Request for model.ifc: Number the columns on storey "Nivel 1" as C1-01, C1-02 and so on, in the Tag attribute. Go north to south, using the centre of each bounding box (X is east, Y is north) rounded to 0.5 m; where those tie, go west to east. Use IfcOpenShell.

First a look at what the model holds.

```python
import ifcopenshell
import ifcopenshell.util.element
import ifcopenshell.util.placement

model = ifcopenshell.open("model.ifc")
print(model.schema)
storey = next(s for s in model.by_type("IfcBuildingStorey") if s.Name == "Nivel 1")
columns = [e for e in ifcopenshell.util.element.get_decomposition(storey) if e.is_a("IfcColumn")]
for e in sorted(columns, key=lambda e: e.id()):
    origin = ifcopenshell.util.placement.get_local_placement(e.ObjectPlacement)[:3, 3]
    print(e.id(), e.Tag, e.Name, origin.round(2) + 0.0, sep=" | ")
```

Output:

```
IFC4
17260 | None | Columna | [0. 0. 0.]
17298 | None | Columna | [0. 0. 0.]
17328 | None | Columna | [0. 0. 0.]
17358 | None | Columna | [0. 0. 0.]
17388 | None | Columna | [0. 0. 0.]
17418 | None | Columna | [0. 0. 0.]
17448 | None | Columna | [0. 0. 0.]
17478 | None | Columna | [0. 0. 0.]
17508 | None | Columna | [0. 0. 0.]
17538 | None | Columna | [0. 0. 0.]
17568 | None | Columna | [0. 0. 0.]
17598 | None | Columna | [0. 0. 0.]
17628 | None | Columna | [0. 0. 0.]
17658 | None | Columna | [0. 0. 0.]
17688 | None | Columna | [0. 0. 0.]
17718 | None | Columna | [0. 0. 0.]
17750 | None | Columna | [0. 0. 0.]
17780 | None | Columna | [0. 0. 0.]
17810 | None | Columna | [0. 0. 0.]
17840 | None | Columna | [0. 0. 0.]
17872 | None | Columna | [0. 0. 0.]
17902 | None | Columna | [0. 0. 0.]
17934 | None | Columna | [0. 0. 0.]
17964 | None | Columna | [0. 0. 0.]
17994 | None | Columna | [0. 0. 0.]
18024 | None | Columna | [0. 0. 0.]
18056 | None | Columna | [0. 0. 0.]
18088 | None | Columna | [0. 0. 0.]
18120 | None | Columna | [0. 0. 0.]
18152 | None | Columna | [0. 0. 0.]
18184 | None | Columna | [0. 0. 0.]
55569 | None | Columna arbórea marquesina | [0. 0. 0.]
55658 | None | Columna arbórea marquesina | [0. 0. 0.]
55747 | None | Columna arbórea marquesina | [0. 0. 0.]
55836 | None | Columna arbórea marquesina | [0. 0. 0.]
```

```python
import ifcopenshell
import ifcopenshell.geom
import ifcopenshell.util.element
import ifcopenshell.util.shape

model = ifcopenshell.open("model.ifc")
settings = ifcopenshell.geom.settings()
settings.set("use-world-coords", True)


def centre(element):
    shape = ifcopenshell.geom.create_shape(settings, element)
    return ifcopenshell.util.shape.get_bbox_centroid(shape.geometry)


storey = next(s for s in model.by_type("IfcBuildingStorey") if s.Name == "Nivel 1")
columns = [e for e in ifcopenshell.util.element.get_decomposition(storey) if e.is_a("IfcColumn")]

# Insertion points can sit at a corner or the storey origin, so sort by the geometry (in metres).
centres = {e: centre(e) for e in columns}
columns.sort(key=lambda e: (-round(centres[e][1] / 0.5), centres[e][0]))

for i, e in enumerate(columns, start=1):
    number = f"C1-{i:02d}"
    e.Tag = number
    print(e.id(), number)

model.write("model_edited.ifc")
```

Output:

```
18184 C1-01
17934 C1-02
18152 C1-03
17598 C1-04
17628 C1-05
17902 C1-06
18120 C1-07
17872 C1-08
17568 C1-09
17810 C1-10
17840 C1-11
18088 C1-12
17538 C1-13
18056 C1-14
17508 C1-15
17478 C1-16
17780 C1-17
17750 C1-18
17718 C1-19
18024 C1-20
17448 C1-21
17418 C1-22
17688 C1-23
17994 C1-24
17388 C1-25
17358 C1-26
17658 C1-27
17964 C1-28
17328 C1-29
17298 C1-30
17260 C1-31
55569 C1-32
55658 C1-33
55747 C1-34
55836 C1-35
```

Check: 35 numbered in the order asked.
